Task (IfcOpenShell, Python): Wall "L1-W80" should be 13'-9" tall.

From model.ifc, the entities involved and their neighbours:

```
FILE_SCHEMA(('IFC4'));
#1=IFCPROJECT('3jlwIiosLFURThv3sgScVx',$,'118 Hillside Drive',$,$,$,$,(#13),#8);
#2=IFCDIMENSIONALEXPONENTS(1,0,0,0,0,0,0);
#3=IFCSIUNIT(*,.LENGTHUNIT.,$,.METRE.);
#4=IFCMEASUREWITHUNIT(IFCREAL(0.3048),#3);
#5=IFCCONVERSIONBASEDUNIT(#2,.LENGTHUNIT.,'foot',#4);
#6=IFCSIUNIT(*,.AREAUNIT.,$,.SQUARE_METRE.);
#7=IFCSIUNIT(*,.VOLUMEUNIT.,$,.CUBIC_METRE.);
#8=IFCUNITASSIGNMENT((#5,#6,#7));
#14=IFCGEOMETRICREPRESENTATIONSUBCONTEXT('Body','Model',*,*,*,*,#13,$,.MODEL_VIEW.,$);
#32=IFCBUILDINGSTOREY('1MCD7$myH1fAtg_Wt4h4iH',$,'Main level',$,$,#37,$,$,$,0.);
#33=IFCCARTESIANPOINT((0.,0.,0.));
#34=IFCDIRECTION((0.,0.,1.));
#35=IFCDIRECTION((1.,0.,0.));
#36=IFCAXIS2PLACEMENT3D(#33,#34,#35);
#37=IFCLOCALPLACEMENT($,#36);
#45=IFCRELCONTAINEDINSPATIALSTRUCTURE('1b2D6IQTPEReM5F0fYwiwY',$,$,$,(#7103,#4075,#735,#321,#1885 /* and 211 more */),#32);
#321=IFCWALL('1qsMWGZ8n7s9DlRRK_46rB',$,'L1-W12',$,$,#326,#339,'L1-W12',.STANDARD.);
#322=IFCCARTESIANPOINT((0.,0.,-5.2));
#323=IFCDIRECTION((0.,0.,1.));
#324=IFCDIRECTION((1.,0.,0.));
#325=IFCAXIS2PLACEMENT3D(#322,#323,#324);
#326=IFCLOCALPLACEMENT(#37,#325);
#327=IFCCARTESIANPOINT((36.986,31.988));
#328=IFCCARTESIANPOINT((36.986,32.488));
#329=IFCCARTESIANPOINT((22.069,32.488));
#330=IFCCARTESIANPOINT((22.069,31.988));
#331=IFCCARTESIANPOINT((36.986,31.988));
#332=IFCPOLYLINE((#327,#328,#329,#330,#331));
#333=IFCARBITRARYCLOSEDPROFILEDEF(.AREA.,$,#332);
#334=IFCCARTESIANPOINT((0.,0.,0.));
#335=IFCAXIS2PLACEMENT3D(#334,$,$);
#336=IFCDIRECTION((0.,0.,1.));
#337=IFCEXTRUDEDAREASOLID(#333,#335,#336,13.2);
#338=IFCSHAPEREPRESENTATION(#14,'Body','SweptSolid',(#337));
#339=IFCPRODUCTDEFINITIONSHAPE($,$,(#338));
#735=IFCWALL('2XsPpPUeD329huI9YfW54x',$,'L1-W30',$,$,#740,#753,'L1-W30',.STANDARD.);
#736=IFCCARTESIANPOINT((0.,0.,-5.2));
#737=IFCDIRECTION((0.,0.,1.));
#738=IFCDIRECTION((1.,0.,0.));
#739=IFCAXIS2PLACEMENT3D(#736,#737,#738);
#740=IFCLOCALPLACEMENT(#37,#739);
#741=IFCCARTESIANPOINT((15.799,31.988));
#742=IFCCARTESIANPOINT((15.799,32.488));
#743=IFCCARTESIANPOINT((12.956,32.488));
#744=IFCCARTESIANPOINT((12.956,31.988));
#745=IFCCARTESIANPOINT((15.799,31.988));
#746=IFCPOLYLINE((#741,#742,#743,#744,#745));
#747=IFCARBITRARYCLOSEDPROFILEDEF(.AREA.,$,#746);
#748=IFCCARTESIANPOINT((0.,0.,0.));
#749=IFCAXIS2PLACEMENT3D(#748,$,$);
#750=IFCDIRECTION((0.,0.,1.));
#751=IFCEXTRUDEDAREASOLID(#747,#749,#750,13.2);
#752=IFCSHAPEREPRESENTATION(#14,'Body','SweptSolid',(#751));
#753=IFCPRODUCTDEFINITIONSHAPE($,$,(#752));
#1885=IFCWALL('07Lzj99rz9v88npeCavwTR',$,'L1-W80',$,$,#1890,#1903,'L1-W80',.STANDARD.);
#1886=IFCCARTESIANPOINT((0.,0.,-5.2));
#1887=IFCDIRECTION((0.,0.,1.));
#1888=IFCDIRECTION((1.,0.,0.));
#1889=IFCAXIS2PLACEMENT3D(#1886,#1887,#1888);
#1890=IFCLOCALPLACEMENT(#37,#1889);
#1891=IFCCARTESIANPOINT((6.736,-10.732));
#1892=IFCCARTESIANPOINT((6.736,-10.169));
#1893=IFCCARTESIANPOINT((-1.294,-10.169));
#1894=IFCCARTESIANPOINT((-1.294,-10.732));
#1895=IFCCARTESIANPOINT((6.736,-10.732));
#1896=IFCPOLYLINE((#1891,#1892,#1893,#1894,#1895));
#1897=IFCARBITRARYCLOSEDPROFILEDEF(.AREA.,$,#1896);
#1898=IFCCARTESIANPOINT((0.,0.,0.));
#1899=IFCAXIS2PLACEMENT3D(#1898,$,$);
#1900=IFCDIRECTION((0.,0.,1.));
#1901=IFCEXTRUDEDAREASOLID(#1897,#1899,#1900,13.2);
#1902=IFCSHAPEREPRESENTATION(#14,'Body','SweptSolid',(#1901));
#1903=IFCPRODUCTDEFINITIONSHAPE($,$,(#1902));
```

```python
import ifcopenshell
import ifcopenshell.geom
import ifcopenshell.util.representation
import ifcopenshell.util.shape
import ifcopenshell.util.unit

model = ifcopenshell.open("model.ifc")
unit_scale = ifcopenshell.util.unit.calculate_unit_scale(model)
settings = ifcopenshell.geom.settings()


def volume(element):
    """Net volume in cubic metres, openings subtracted."""
    shape = ifcopenshell.geom.create_shape(settings, element)
    return ifcopenshell.util.shape.get_volume(shape.geometry)


wall = model.by_guid("07Lzj99rz9v88npeCavwTR")
before = volume(wall)

body = ifcopenshell.util.representation.get_representation(wall, "Model", "Body")
solid = body.Items[0]
old_height = solid.Depth
solid.Depth = 165 * 0.0254 / unit_scale
after = volume(wall)

print(f"height {old_height:g} -> {solid.Depth:g}, volume {before:.3f} -> {after:.3f} m3")

model.write("model_v2.ifc")
```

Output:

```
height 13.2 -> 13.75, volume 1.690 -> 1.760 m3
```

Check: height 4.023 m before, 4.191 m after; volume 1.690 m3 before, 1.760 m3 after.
